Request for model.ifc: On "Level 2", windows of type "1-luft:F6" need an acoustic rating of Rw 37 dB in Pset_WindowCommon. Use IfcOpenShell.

First a look at what the model holds.

```python
import ifcopenshell
import ifcopenshell.util.element

model = ifcopenshell.open("model.ifc")
print(model.schema)
storey = next(s for s in model.by_type("IfcBuildingStorey") if s.Name == "Level 2")
windows = [e for e in ifcopenshell.util.element.get_decomposition(storey) if e.is_a("IfcWindow")]
seen = {}
for e in windows:
    element_type = ifcopenshell.util.element.get_type(e)
    key = (element_type.Name if element_type != e and element_type else None, ifcopenshell.util.element.get_pset(e, "Pset_WindowCommon", "AcousticRating"))
    seen[key] = seen.get(key, 0) + 1
for (name, value), count in sorted(seen.items(), key=str):
    print(count, "x", name, "|", value)
```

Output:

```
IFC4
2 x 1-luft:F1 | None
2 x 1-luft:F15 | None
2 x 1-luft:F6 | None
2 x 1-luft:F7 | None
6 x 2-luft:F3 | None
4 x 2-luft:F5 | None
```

```python
import ifcopenshell
import ifcopenshell.api.pset
import ifcopenshell.util.element

model = ifcopenshell.open("model.ifc")

storey = next(s for s in model.by_type("IfcBuildingStorey") if s.Name == "Level 2")
windows = [e for e in ifcopenshell.util.element.get_decomposition(storey) if e.is_a("IfcWindow")]

count = 0
for e in windows:
    element_type = ifcopenshell.util.element.get_type(e)
    if element_type in (None, e) or element_type.Name != "1-luft:F6":
        continue
    # add_pset returns the element's existing set when there is one.
    pset = ifcopenshell.api.pset.add_pset(model, product=e, name="Pset_WindowCommon")
    ifcopenshell.api.pset.edit_pset(model, pset=pset, properties={"AcousticRating": "Rw 37 dB"})
    count += 1

print(count, "windows updated")

model.write("model_v2.ifc")
```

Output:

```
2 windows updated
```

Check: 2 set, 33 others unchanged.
